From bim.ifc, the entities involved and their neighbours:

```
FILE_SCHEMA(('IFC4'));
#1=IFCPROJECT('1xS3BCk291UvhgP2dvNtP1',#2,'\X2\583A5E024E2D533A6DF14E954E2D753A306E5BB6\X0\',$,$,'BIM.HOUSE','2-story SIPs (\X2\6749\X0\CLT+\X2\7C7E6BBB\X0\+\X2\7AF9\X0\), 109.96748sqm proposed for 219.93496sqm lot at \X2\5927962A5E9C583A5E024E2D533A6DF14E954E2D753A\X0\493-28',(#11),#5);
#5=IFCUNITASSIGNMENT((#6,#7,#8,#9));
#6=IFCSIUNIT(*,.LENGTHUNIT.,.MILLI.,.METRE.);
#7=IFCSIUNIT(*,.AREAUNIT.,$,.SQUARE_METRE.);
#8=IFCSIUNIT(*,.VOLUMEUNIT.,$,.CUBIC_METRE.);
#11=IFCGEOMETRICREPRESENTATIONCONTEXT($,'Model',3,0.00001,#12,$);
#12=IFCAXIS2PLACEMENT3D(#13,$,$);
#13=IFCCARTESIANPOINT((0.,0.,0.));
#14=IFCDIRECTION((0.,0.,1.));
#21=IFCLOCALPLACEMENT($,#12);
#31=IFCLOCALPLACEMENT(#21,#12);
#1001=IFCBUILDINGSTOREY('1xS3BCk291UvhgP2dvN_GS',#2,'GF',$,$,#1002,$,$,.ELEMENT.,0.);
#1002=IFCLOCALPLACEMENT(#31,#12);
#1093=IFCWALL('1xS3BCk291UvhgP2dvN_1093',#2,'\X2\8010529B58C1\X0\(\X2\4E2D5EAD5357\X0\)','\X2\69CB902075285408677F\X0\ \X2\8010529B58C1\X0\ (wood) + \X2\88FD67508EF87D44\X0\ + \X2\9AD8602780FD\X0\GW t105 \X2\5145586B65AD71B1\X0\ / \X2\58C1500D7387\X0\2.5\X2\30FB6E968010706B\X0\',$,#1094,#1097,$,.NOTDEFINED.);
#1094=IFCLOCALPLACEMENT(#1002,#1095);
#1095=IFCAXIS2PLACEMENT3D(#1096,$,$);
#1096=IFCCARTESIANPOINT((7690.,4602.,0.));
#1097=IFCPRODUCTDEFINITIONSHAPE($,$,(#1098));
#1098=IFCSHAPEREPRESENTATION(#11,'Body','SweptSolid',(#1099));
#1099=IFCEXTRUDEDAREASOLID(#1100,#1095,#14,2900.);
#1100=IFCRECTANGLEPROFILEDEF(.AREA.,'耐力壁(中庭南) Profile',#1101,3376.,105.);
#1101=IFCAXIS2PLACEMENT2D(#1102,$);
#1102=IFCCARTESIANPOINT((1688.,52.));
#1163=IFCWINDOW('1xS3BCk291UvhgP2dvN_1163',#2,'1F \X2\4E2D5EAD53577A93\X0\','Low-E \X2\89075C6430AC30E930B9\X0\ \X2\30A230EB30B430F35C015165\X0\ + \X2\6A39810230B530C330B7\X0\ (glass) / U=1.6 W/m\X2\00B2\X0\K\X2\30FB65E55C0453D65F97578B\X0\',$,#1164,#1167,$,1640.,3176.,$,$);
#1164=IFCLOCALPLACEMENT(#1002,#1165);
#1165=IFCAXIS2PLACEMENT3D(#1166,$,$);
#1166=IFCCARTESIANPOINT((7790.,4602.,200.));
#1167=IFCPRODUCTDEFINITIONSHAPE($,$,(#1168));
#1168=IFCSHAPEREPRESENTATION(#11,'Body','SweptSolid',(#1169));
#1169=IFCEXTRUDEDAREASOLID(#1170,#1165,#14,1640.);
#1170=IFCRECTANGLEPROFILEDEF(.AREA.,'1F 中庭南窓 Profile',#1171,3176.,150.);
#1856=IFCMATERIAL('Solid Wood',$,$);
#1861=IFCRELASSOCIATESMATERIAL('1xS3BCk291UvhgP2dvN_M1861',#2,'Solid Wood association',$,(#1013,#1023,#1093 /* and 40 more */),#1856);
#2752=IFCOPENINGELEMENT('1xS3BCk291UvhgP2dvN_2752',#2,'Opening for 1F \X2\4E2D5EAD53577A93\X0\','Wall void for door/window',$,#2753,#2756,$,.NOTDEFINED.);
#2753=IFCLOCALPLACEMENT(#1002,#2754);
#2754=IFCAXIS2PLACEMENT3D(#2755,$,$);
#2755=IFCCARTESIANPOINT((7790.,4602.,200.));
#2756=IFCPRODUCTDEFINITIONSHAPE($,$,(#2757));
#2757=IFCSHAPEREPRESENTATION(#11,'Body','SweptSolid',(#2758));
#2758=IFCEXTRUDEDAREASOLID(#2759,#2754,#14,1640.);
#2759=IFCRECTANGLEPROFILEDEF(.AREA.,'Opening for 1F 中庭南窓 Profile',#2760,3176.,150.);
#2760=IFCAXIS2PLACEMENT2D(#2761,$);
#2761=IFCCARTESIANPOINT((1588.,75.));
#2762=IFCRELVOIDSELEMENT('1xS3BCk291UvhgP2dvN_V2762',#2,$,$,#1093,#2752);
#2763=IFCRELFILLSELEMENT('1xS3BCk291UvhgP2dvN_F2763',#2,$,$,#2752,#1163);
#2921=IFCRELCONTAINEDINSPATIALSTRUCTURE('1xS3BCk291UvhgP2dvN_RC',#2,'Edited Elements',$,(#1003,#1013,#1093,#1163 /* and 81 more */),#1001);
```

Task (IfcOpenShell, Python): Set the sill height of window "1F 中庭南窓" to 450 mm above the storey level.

```python
import numpy as np
import ifcopenshell
import ifcopenshell.api.geometry
import ifcopenshell.geom
import ifcopenshell.util.element
import ifcopenshell.util.placement
import ifcopenshell.util.shape
import ifcopenshell.util.unit

model = ifcopenshell.open("bim.ifc")
unit_scale = ifcopenshell.util.unit.calculate_unit_scale(model)

window = model.by_guid("1xS3BCk291UvhgP2dvN_1163")
opening = window.FillsVoids[0].RelatingOpeningElement
storey = ifcopenshell.util.element.get_container(window, ifc_class="IfcBuildingStorey")
level = ifcopenshell.util.placement.get_local_placement(storey.ObjectPlacement)[2, 3]

# The opening's origin need not be at the sill, so measure its lowest point.
shape = ifcopenshell.geom.create_shape(ifcopenshell.geom.settings(), opening)
bottom = ifcopenshell.util.shape.get_shape_bottom_elevation(shape, shape.geometry) / unit_scale
dz = level + 0.45 / unit_scale - bottom

shift = np.array([0.0, 0.0, dz])
# The window is not placed relative to its opening, so move both.
for product in (opening, window):
    matrix = ifcopenshell.util.placement.get_local_placement(product.ObjectPlacement)
    matrix[:3, 3] += shift
    ifcopenshell.api.geometry.edit_object_placement(model, product=product, matrix=matrix, is_si=False)

print(f"moved by {dz * unit_scale:+.3f} m")

model.write("bim_updated.ifc")
```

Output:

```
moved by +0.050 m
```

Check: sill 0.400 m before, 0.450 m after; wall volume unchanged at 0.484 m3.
